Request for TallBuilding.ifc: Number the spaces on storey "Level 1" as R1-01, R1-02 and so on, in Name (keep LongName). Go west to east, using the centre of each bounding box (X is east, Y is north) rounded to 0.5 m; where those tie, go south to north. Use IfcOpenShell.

First a look at what the model holds.

```python
import ifcopenshell
import ifcopenshell.util.element
import ifcopenshell.util.placement

model = ifcopenshell.open("TallBuilding.ifc")
print(model.schema)
storey = next(s for s in model.by_type("IfcBuildingStorey") if s.Name == "Level 1")
spaces = [e for e in ifcopenshell.util.element.get_decomposition(storey) if e.is_a("IfcSpace")]
for e in sorted(spaces, key=lambda e: e.id()):
    origin = ifcopenshell.util.placement.get_local_placement(e.ObjectPlacement)[:3, 3]
    print(e.id(), e.Name, e.LongName, origin.round(2) + 0.0, sep=" | ")
```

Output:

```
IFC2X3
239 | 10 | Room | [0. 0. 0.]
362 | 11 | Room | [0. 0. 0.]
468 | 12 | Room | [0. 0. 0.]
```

```python
import ifcopenshell
import ifcopenshell.geom
import ifcopenshell.util.element
import ifcopenshell.util.shape

model = ifcopenshell.open("TallBuilding.ifc")
settings = ifcopenshell.geom.settings()
settings.set("use-world-coords", True)


def centre(element):
    shape = ifcopenshell.geom.create_shape(settings, element)
    return ifcopenshell.util.shape.get_bbox_centroid(shape.geometry)


storey = next(s for s in model.by_type("IfcBuildingStorey") if s.Name == "Level 1")
spaces = [e for e in ifcopenshell.util.element.get_decomposition(storey) if e.is_a("IfcSpace")]

# Insertion points can sit at a corner or the storey origin, so sort by the geometry (in metres).
centres = {e: centre(e) for e in spaces}
spaces.sort(key=lambda e: (round(centres[e][0] / 0.5), centres[e][1]))

for i, e in enumerate(spaces, start=1):
    number = f"R1-{i:02d}"
    e.Name = number
    print(e.id(), number)

model.write("TallBuilding_updated.ifc")
```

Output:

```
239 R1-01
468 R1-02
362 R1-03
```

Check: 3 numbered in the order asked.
